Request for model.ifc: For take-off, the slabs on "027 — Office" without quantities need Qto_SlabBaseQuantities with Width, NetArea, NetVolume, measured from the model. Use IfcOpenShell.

First a look at what the model holds.

```python
import ifcopenshell
import ifcopenshell.util.element
import ifcopenshell.util.unit

model = ifcopenshell.open("model.ifc")
print(model.schema)
for unit_type in ("LENGTHUNIT", "AREAUNIT", "VOLUMEUNIT"):
    print(unit_type, ifcopenshell.util.unit.calculate_unit_scale(model, unit_type))
storey = next(s for s in model.by_type("IfcBuildingStorey") if s.Name == "027 — Office")
slabs = [e for e in ifcopenshell.util.element.get_decomposition(storey) if e.is_a("IfcSlab")]
for e in sorted(slabs, key=lambda e: e.id()):
    print(e.id(), e.is_a(), e.Name, list(ifcopenshell.util.element.get_psets(e, qtos_only=True)), sep=" | ")
```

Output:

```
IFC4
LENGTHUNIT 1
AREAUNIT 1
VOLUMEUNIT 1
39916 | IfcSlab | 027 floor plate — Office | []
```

```python
import ifcopenshell
import ifcopenshell.api.pset
import ifcopenshell.geom
import ifcopenshell.util.element
import ifcopenshell.util.shape
import ifcopenshell.util.unit

model = ifcopenshell.open("model.ifc")
unit_scale = ifcopenshell.util.unit.calculate_unit_scale(model)
area_scale = ifcopenshell.util.unit.calculate_unit_scale(model, "AREAUNIT")
volume_scale = ifcopenshell.util.unit.calculate_unit_scale(model, "VOLUMEUNIT")
settings = ifcopenshell.geom.settings()

storey = next(s for s in model.by_type("IfcBuildingStorey") if s.Name == "027 — Office")
slabs = [e for e in ifcopenshell.util.element.get_decomposition(storey) if e.is_a("IfcSlab")]

for e in sorted(slabs, key=lambda e: e.id()):
    if ifcopenshell.util.element.get_psets(e, qtos_only=True, should_inherit=False):
        continue
    # Geometry comes back in metres, in the element's own axes.
    shape = ifcopenshell.geom.create_shape(settings, e)
    values = {
        "Width": ifcopenshell.util.shape.get_z(shape.geometry) / unit_scale,
        "NetArea": ifcopenshell.util.shape.get_footprint_area(shape.geometry) / area_scale,
        "NetVolume": ifcopenshell.util.shape.get_volume(shape.geometry) / volume_scale,
    }
    qto = ifcopenshell.api.pset.add_qto(model, product=e, name="Qto_SlabBaseQuantities")
    ifcopenshell.api.pset.edit_qto(model, qto=qto, properties=values)
    print(e.id(), {k: round(v, 3) for k, v in values.items()})

model.write("model_v2.ifc")
```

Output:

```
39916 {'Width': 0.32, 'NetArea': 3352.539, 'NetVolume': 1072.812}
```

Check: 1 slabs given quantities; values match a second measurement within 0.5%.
